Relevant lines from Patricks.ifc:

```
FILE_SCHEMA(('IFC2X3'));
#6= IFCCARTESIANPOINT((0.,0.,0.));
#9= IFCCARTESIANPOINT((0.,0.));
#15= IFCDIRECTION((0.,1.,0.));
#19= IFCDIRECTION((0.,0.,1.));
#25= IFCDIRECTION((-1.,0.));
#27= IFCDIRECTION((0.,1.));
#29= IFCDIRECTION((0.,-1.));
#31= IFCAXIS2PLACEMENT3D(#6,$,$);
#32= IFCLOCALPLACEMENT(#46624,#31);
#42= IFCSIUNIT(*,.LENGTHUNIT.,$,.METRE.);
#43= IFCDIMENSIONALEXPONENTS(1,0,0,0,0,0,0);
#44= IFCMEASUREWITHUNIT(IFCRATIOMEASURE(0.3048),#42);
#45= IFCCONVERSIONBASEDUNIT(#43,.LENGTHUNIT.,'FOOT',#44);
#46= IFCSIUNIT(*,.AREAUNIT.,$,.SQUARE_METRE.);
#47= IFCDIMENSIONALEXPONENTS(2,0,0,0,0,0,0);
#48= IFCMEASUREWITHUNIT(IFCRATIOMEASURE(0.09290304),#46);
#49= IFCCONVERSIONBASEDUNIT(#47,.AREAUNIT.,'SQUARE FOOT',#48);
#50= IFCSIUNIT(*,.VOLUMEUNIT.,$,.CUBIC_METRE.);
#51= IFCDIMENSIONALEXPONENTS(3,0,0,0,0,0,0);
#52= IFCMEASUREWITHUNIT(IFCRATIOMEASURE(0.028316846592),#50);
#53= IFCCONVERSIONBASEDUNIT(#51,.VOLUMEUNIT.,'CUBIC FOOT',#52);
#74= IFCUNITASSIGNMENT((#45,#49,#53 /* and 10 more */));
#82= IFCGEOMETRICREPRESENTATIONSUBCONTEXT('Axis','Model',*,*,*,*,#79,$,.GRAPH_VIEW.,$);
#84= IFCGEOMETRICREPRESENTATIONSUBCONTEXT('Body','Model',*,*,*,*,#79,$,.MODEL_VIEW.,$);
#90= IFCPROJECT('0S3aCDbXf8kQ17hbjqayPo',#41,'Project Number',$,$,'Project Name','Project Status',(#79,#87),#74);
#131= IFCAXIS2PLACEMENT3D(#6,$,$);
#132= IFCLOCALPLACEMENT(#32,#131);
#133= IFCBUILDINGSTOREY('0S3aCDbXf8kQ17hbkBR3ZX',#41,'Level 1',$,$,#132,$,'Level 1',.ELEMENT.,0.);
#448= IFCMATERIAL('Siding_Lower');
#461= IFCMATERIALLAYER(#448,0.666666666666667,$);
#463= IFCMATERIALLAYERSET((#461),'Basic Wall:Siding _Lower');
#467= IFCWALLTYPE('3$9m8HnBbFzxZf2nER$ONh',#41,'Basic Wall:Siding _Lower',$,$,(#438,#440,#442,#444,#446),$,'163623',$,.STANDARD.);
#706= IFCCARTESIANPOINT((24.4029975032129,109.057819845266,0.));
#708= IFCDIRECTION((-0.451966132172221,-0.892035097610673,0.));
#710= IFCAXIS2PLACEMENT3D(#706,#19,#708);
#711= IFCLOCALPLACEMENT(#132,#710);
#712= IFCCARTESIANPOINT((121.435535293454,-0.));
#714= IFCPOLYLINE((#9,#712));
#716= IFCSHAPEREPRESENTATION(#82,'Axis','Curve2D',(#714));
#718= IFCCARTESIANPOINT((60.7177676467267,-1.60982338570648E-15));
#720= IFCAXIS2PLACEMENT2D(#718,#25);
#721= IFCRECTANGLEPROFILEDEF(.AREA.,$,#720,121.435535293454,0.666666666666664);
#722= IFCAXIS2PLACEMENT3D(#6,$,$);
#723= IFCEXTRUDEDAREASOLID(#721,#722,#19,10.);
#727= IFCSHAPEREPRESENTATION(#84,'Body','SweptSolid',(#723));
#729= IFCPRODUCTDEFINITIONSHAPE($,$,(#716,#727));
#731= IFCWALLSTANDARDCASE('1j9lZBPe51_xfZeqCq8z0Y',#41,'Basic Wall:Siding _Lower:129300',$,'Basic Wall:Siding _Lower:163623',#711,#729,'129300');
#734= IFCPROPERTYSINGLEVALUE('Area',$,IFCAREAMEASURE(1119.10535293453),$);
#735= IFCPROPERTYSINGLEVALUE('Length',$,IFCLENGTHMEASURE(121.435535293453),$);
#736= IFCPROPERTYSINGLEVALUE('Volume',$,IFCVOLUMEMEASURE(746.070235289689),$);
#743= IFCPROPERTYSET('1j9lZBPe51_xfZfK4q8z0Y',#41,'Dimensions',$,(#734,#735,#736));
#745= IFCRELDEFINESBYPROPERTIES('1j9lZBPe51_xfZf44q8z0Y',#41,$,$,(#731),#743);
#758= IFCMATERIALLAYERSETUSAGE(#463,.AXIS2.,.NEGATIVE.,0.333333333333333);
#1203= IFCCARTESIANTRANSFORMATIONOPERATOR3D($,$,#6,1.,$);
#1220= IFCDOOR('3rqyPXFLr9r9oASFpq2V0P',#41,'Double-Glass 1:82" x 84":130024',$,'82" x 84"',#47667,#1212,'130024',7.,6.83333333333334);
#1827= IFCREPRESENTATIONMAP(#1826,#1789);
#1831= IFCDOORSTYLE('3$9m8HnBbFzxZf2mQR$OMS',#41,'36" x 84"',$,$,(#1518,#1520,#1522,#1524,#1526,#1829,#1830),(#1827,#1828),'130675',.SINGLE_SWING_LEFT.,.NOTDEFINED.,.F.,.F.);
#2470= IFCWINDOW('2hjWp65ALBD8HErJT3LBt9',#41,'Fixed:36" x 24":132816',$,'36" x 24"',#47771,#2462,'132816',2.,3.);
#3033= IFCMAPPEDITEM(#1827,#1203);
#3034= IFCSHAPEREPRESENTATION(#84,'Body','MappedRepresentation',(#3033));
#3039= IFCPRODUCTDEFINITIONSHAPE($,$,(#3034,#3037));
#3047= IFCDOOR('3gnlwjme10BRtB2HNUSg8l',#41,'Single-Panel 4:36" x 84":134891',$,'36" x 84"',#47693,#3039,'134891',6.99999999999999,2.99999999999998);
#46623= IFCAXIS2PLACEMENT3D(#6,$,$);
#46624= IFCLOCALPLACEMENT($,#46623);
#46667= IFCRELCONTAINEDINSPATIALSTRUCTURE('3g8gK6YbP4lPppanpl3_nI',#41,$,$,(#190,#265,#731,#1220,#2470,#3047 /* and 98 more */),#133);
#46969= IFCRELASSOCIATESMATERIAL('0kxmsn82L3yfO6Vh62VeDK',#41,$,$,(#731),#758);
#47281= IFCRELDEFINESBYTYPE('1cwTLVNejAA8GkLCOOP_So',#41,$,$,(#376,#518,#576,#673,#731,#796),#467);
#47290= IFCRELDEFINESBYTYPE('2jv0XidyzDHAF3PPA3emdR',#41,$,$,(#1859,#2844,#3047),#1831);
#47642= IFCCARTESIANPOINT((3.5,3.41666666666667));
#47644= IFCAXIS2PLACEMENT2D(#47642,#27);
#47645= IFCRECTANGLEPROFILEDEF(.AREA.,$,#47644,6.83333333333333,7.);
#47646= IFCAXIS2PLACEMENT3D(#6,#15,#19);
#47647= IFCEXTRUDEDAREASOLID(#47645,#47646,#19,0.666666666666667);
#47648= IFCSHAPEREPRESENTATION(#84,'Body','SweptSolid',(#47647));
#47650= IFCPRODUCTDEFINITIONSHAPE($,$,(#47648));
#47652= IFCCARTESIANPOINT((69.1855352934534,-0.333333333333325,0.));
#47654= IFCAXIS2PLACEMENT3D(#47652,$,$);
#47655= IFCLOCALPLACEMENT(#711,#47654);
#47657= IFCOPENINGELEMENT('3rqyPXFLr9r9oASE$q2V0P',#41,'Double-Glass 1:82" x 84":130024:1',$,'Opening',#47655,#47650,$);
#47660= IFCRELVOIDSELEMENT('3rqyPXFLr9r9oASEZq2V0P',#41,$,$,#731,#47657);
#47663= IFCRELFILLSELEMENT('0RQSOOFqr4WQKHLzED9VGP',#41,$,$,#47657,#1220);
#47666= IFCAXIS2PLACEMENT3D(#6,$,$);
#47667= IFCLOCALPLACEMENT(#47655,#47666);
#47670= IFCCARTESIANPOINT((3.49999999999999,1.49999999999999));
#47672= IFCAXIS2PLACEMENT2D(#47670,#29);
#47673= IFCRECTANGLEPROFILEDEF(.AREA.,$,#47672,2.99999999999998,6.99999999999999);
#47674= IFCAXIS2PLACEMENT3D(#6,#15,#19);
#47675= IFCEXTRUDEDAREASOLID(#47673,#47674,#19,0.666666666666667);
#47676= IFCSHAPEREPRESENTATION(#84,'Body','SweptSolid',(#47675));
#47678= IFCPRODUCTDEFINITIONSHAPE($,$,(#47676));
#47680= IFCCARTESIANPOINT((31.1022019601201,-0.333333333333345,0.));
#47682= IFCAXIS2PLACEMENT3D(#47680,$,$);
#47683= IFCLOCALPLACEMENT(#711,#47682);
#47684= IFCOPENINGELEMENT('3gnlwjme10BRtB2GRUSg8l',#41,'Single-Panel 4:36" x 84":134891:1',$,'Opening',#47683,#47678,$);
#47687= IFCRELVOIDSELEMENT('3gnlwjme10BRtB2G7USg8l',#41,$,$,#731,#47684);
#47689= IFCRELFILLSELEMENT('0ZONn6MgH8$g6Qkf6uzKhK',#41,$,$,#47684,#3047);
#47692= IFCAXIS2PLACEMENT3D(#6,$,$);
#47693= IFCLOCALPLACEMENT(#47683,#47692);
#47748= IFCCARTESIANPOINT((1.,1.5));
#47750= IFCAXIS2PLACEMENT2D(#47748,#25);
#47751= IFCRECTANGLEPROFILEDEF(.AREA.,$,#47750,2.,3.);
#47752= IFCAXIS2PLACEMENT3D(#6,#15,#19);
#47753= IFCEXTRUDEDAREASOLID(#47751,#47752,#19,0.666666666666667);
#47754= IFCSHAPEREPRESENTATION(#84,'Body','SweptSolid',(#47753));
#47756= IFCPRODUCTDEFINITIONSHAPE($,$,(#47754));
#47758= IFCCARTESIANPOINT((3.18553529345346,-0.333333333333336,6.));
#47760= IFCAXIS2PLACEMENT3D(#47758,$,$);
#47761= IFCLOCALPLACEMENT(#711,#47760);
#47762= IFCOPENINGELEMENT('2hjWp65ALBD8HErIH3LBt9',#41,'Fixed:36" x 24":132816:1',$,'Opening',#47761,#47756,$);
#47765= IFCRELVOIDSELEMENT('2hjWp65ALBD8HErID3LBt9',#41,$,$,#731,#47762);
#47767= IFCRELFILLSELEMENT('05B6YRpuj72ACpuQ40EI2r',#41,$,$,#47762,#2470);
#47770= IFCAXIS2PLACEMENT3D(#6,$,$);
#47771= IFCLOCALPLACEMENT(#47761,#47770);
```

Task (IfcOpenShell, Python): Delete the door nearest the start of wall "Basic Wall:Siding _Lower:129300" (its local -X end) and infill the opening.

```python
import ifcopenshell
import ifcopenshell.api.feature
import ifcopenshell.api.pset
import ifcopenshell.api.root
import ifcopenshell.geom
import ifcopenshell.util.element
import ifcopenshell.util.shape
import ifcopenshell.util.unit

model = ifcopenshell.open("Patricks.ifc")
area_scale = ifcopenshell.util.unit.calculate_unit_scale(model, "AREAUNIT")
volume_scale = ifcopenshell.util.unit.calculate_unit_scale(model, "VOLUMEUNIT")
settings = ifcopenshell.geom.settings()


def volume(element):
    """Net volume in cubic metres, openings subtracted."""
    shape = ifcopenshell.geom.create_shape(settings, element)
    return ifcopenshell.util.shape.get_volume(shape.geometry)


door = model.by_guid("3gnlwjme10BRtB2HNUSg8l")
opening = door.FillsVoids[0].RelatingOpeningElement
wall = opening.VoidsElements[0].RelatingBuildingElement
before = volume(wall)

ifcopenshell.api.root.remove_product(model, product=door)
ifcopenshell.api.feature.remove_feature(model, feature=opening)

after = volume(wall)
thickness = 0.2032  # wall thickness in metres

# Update the wall's stored quantities.
pset = model.by_id(ifcopenshell.util.element.get_pset(wall, "Dimensions", should_inherit=False)["id"])
ifcopenshell.api.pset.edit_pset(model, pset=pset, properties={
    "Area": model.create_entity("IfcAreaMeasure", after / thickness / area_scale),
    "Volume": model.create_entity("IfcVolumeMeasure", after / volume_scale),
})

print(f"wall volume {before:.3f} -> {after:.3f} m3")

model.write("Patricks_rev.ifc")
```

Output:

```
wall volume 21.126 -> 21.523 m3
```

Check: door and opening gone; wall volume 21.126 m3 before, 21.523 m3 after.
